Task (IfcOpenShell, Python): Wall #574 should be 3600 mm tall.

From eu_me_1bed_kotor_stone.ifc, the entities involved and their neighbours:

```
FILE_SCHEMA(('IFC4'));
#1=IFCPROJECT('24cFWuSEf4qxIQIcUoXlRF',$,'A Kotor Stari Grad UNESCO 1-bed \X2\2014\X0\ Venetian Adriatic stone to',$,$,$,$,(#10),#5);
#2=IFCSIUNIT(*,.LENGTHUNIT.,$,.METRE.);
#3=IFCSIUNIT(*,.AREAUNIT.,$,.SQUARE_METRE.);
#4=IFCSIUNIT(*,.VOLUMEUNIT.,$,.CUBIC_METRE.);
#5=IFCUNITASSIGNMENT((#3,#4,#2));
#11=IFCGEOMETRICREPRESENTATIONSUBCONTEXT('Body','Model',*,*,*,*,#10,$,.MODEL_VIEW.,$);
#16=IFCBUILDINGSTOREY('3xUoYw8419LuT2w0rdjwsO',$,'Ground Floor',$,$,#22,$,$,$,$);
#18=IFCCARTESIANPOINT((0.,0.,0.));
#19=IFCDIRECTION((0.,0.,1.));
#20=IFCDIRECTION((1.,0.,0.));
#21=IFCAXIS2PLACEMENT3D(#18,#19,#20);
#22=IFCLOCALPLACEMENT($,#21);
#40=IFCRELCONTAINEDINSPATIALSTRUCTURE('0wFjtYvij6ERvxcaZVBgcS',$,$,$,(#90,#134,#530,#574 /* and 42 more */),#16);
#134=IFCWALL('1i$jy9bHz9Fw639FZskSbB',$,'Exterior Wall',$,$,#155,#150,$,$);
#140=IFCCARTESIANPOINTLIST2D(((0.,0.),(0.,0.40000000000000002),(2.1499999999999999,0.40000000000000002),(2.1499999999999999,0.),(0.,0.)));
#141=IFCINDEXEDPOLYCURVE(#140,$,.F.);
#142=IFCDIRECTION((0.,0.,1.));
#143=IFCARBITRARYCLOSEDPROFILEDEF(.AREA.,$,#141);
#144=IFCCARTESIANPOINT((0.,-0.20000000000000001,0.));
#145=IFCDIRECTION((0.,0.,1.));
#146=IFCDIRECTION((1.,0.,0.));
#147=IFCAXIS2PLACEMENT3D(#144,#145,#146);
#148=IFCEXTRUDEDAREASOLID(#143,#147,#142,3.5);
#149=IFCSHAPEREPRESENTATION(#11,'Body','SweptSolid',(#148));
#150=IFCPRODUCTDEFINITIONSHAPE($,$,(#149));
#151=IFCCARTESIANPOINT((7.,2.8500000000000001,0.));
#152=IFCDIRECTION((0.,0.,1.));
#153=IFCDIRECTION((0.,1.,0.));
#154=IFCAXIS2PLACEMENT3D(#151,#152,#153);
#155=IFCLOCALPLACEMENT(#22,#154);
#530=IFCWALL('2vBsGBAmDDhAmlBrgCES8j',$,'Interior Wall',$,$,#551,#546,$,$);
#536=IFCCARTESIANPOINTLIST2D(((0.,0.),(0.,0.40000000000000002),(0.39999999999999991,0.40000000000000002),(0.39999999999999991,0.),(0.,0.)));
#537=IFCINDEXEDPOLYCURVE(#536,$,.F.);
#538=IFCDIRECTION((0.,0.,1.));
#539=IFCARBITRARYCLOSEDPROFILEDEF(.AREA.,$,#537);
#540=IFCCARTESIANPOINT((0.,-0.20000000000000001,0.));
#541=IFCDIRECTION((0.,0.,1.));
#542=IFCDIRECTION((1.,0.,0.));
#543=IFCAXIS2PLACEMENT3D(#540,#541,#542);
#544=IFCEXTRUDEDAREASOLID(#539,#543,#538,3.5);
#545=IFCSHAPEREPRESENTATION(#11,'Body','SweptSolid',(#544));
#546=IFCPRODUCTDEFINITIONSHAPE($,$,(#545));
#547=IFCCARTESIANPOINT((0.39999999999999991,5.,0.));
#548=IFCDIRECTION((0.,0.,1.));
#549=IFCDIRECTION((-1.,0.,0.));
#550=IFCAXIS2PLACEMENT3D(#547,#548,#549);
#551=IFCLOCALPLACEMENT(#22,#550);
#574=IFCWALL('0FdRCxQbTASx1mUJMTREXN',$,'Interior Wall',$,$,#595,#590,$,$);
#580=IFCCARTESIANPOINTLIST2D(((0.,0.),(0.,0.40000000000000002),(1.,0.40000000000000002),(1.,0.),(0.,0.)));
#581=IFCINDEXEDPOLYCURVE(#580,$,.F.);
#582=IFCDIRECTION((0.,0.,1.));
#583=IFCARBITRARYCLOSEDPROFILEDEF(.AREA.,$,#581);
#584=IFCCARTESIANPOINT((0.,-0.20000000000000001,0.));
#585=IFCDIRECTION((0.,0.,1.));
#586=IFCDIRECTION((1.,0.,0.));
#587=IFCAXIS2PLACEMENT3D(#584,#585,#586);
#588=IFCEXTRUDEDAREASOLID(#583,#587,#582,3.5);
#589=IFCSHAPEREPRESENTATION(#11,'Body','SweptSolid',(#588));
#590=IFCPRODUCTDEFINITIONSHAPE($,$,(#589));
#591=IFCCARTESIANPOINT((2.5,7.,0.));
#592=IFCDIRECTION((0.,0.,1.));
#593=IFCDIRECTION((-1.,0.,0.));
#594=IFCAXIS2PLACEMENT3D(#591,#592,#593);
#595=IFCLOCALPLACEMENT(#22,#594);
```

```python
import ifcopenshell
import ifcopenshell.geom
import ifcopenshell.util.representation
import ifcopenshell.util.shape

model = ifcopenshell.open("eu_me_1bed_kotor_stone.ifc")
settings = ifcopenshell.geom.settings()


def volume(element):
    """Net volume in cubic metres, openings subtracted."""
    shape = ifcopenshell.geom.create_shape(settings, element)
    return ifcopenshell.util.shape.get_volume(shape.geometry)


wall = model.by_guid("0FdRCxQbTASx1mUJMTREXN")
before = volume(wall)

body = ifcopenshell.util.representation.get_representation(wall, "Model", "Body")
solid = body.Items[0]
old_height = solid.Depth
solid.Depth = 3.6
after = volume(wall)

print(f"height {old_height:g} -> {solid.Depth:g}, volume {before:.3f} -> {after:.3f} m3")

model.write("eu_me_1bed_kotor_stone-out.ifc")
```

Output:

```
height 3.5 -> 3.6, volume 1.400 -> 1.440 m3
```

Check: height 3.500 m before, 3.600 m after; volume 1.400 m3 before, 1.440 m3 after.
